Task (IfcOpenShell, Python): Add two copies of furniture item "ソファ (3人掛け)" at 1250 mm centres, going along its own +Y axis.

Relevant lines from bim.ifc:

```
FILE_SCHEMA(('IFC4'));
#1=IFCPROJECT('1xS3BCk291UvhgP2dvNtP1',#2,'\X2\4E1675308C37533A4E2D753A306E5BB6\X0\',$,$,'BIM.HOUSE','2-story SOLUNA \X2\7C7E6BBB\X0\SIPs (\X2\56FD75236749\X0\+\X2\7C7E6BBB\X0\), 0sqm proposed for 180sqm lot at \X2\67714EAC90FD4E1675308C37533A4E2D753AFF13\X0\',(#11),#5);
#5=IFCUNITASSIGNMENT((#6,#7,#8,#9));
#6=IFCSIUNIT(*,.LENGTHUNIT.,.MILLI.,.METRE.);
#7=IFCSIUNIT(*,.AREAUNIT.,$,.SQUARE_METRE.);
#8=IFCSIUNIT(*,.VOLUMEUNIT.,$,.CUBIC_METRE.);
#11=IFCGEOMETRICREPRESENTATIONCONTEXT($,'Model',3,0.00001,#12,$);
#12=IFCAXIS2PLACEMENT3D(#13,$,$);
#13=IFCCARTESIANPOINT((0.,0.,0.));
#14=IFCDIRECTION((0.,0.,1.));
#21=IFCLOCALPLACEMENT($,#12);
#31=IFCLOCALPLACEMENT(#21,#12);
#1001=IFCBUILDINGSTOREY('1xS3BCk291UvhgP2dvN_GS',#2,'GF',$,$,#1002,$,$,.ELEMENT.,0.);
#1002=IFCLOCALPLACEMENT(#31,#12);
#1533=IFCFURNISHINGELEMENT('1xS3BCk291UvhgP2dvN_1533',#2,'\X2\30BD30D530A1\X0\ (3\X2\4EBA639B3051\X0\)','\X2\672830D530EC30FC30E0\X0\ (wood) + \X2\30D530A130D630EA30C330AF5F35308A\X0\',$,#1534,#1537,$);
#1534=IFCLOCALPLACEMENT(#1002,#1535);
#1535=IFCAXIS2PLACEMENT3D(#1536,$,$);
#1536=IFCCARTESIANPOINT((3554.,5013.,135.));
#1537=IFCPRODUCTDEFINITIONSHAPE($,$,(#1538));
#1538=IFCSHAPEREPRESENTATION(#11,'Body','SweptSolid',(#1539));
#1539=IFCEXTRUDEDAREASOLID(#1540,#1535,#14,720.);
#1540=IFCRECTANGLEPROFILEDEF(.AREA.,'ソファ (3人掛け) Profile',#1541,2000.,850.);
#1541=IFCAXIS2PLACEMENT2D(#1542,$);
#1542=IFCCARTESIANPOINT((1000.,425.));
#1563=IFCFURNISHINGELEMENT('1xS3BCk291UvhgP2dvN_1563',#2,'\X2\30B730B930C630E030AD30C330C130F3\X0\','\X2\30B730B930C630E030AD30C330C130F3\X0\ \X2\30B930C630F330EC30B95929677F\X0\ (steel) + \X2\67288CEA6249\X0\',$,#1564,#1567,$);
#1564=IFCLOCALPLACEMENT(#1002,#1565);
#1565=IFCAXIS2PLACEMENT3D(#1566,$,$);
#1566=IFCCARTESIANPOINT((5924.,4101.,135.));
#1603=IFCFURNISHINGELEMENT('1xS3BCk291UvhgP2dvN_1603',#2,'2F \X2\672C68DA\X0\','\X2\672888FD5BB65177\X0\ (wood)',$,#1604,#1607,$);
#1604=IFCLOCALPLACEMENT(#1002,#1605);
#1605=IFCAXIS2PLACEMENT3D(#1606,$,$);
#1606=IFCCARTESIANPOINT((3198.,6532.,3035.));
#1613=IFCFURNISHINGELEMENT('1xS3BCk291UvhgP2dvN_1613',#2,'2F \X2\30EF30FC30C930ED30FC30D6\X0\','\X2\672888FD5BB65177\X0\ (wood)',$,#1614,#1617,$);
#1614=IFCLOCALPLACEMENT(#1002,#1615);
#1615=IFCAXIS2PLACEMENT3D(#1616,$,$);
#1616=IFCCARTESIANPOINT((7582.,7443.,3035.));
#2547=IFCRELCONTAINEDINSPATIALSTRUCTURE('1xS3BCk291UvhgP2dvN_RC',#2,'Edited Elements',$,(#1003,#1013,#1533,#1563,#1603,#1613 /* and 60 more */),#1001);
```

```python
import ifcopenshell
import ifcopenshell.api.geometry
import ifcopenshell.api.root
import ifcopenshell.util.element
import ifcopenshell.util.placement
import ifcopenshell.util.unit

model = ifcopenshell.open("bim.ifc")
unit_scale = ifcopenshell.util.unit.calculate_unit_scale(model)


def reuse_history(source, copy):
    """copy_class also copies each property set's owner history, people and application; keep the originals."""
    for rel in copy.IsDefinedBy:
        if rel.is_a("IfcRelDefinesByProperties") and (history := rel.RelatingPropertyDefinition.OwnerHistory):
            rel.RelatingPropertyDefinition.OwnerHistory = source.OwnerHistory
            ifcopenshell.util.element.remove_deep2(model, history)


source = model.by_guid("1xS3BCk291UvhgP2dvN_1533")
base = ifcopenshell.util.placement.get_local_placement(source.ObjectPlacement)
step = base[:3, 1] * 1.25 / unit_scale

for i in range(1, 3):
    copy = ifcopenshell.api.root.copy_class(model, product=source)
    copy.Representation = ifcopenshell.util.element.copy_deep(
        model, source.Representation, exclude=["IfcGeometricRepresentationContext", "IfcRepresentationMap"]
    )
    reuse_history(source, copy)
    matrix = base.copy()
    matrix[:3, 3] += i * step
    print("added at", matrix[:3, 3].round(3) + 0.0)
    ifcopenshell.api.geometry.edit_object_placement(model, product=copy, matrix=matrix, is_si=False)

model.write("bim_v2.ifc")
```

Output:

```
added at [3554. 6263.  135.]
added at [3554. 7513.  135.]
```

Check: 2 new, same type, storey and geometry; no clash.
